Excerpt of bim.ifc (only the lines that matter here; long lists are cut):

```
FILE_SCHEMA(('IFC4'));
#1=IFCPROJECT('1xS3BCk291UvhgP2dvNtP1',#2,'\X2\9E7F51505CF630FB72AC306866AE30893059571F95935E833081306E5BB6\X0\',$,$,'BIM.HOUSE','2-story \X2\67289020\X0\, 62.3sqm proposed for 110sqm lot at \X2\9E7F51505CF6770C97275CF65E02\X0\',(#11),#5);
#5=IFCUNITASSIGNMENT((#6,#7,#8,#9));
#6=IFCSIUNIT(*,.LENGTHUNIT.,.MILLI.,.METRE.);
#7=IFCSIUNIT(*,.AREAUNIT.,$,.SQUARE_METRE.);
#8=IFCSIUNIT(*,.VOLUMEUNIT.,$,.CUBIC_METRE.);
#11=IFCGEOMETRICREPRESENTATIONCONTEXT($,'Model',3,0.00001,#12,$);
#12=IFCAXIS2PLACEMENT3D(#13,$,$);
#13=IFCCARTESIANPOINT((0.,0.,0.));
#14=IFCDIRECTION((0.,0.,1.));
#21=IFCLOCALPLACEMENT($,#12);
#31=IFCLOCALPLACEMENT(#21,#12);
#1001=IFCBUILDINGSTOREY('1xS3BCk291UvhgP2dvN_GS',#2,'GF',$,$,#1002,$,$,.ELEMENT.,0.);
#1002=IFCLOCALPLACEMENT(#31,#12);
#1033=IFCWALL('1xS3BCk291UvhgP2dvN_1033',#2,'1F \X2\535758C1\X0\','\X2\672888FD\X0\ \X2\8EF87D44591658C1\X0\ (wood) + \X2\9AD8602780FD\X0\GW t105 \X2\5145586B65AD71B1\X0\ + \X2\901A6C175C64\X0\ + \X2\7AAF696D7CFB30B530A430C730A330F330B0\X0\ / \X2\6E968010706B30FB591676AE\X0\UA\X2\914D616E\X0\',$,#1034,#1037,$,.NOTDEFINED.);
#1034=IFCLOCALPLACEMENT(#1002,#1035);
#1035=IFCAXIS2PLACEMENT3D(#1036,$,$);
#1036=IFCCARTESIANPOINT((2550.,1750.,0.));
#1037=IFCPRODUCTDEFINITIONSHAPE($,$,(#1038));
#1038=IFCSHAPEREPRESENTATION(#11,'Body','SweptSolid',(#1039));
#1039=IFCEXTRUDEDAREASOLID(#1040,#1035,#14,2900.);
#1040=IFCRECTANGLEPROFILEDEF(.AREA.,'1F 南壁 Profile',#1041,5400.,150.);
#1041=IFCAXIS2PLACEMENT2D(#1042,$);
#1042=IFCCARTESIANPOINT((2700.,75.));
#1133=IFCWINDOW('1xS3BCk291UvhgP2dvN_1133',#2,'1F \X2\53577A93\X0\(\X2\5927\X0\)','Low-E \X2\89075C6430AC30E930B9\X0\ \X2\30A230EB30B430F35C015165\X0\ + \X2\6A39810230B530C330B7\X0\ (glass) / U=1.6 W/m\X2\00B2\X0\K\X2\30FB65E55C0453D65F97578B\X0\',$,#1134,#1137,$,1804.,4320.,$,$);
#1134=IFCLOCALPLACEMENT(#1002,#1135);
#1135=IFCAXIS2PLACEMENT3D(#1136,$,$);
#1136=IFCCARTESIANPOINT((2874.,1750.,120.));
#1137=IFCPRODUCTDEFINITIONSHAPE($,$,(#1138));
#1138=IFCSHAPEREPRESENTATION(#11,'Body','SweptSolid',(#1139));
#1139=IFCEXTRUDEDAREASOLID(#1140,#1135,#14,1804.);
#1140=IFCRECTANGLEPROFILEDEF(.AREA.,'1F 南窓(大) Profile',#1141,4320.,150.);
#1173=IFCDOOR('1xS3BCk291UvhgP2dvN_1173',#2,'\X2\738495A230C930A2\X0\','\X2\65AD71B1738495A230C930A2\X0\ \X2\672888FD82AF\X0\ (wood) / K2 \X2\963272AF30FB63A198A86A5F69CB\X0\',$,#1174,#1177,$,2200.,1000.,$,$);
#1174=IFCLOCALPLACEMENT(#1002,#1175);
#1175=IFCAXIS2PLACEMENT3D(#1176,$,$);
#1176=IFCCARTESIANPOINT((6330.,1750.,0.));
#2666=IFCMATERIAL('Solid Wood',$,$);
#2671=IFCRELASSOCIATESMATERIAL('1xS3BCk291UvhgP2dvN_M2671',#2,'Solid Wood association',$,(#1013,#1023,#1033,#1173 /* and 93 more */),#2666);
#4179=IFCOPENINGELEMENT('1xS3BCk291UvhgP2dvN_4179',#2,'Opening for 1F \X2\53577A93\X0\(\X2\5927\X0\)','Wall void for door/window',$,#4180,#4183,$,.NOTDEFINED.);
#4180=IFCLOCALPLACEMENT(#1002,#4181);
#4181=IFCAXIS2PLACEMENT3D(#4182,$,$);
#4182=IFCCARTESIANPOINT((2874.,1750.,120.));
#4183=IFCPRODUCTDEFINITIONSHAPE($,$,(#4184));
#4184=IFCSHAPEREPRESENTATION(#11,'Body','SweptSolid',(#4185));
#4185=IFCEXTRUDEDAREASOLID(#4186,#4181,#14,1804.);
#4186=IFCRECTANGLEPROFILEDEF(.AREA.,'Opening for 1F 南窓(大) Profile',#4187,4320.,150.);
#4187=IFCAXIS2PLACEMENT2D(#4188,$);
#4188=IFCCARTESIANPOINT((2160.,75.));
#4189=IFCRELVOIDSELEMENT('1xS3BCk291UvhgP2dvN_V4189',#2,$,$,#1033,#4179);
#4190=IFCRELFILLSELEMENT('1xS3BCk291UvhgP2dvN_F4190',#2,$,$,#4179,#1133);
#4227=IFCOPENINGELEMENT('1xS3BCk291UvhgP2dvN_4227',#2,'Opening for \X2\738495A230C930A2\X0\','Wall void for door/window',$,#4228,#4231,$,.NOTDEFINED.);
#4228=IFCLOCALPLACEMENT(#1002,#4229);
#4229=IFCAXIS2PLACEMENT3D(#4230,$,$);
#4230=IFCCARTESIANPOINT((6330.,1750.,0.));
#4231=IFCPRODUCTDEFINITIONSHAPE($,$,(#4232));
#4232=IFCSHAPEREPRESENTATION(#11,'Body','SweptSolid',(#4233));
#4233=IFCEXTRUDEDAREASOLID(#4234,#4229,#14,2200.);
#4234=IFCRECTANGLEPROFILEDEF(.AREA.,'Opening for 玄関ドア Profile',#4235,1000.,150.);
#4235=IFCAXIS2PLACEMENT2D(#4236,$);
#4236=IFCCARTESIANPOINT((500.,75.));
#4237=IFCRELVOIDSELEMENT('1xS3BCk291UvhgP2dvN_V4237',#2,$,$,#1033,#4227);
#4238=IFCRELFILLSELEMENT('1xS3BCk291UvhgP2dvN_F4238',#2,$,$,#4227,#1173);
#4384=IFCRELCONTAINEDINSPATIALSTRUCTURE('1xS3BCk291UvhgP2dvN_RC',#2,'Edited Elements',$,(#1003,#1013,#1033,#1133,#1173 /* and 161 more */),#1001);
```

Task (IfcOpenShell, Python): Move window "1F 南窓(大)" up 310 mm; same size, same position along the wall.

```python
import numpy as np
import ifcopenshell
import ifcopenshell.api.geometry
import ifcopenshell.util.placement
import ifcopenshell.util.unit

model = ifcopenshell.open("bim.ifc")
unit_scale = ifcopenshell.util.unit.calculate_unit_scale(model)

window = model.by_guid("1xS3BCk291UvhgP2dvN_1133")
opening = window.FillsVoids[0].RelatingOpeningElement
dz = 0.31 / unit_scale

shift = np.array([0.0, 0.0, dz])
# The window is not placed relative to its opening, so move both.
for product in (opening, window):
    matrix = ifcopenshell.util.placement.get_local_placement(product.ObjectPlacement)
    matrix[:3, 3] += shift
    ifcopenshell.api.geometry.edit_object_placement(model, product=product, matrix=matrix, is_si=False)

print(f"moved by {dz * unit_scale:+.3f} m")

model.write("bim_updated.ifc")
```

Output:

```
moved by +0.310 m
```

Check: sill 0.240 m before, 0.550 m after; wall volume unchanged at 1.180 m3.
